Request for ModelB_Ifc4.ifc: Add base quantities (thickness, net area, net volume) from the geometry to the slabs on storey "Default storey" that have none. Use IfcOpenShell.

First a look at what the model holds.

```python
import ifcopenshell
import ifcopenshell.util.element
import ifcopenshell.util.unit

model = ifcopenshell.open("ModelB_Ifc4.ifc")
print(model.schema)
for unit_type in ("LENGTHUNIT", "AREAUNIT", "VOLUMEUNIT"):
    print(unit_type, ifcopenshell.util.unit.calculate_unit_scale(model, unit_type))
storey = next(s for s in model.by_type("IfcBuildingStorey") if s.Name == "Default storey")
slabs = [e for e in ifcopenshell.util.element.get_decomposition(storey) if e.is_a("IfcSlab")]
for e in sorted(slabs, key=lambda e: e.id()):
    print(e.id(), e.is_a(), e.Name, list(ifcopenshell.util.element.get_psets(e, qtos_only=True)), sep=" | ")
```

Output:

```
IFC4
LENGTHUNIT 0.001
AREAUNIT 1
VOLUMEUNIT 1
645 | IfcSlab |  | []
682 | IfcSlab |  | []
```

```python
import ifcopenshell
import ifcopenshell.api.pset
import ifcopenshell.geom
import ifcopenshell.util.element
import ifcopenshell.util.shape
import ifcopenshell.util.unit

model = ifcopenshell.open("ModelB_Ifc4.ifc")
unit_scale = ifcopenshell.util.unit.calculate_unit_scale(model)
area_scale = ifcopenshell.util.unit.calculate_unit_scale(model, "AREAUNIT")
volume_scale = ifcopenshell.util.unit.calculate_unit_scale(model, "VOLUMEUNIT")
settings = ifcopenshell.geom.settings()

storey = next(s for s in model.by_type("IfcBuildingStorey") if s.Name == "Default storey")
slabs = [e for e in ifcopenshell.util.element.get_decomposition(storey) if e.is_a("IfcSlab")]

for e in sorted(slabs, key=lambda e: e.id()):
    if ifcopenshell.util.element.get_psets(e, qtos_only=True, should_inherit=False):
        continue
    # Geometry comes back in metres, in the element's own axes.
    shape = ifcopenshell.geom.create_shape(settings, e)
    values = {
        "Width": ifcopenshell.util.shape.get_z(shape.geometry) / unit_scale,
        "NetArea": ifcopenshell.util.shape.get_footprint_area(shape.geometry) / area_scale,
        "NetVolume": ifcopenshell.util.shape.get_volume(shape.geometry) / volume_scale,
    }
    qto = ifcopenshell.api.pset.add_qto(model, product=e, name="Qto_SlabBaseQuantities")
    ifcopenshell.api.pset.edit_qto(model, qto=qto, properties=values)
    print(e.id(), {k: round(v, 3) for k, v in values.items()})

model.write("ModelB_Ifc4_v2.ifc")
```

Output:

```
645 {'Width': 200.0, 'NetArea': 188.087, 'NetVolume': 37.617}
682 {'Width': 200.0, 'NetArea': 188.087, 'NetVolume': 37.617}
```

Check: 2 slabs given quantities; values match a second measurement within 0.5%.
